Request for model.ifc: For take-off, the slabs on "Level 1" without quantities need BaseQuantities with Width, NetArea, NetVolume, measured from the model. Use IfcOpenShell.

First a look at what the model holds.

```python
import ifcopenshell
import ifcopenshell.util.element
import ifcopenshell.util.unit

model = ifcopenshell.open("model.ifc")
print(model.schema)
for unit_type in ("LENGTHUNIT", "AREAUNIT", "VOLUMEUNIT"):
    print(unit_type, ifcopenshell.util.unit.calculate_unit_scale(model, unit_type))
storey = next(s for s in model.by_type("IfcBuildingStorey") if s.Name == "Level 1")
slabs = [e for e in ifcopenshell.util.element.get_decomposition(storey) if e.is_a("IfcSlab")]
for e in sorted(slabs, key=lambda e: e.id()):
    print(e.id(), e.is_a(), e.Name, list(ifcopenshell.util.element.get_psets(e, qtos_only=True)), sep=" | ")
```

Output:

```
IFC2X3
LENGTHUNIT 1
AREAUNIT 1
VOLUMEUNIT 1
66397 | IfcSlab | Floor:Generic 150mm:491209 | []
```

```python
import ifcopenshell
import ifcopenshell.api.pset
import ifcopenshell.geom
import ifcopenshell.util.element
import ifcopenshell.util.shape
import ifcopenshell.util.unit

model = ifcopenshell.open("model.ifc")
unit_scale = ifcopenshell.util.unit.calculate_unit_scale(model)
area_scale = ifcopenshell.util.unit.calculate_unit_scale(model, "AREAUNIT")
volume_scale = ifcopenshell.util.unit.calculate_unit_scale(model, "VOLUMEUNIT")
settings = ifcopenshell.geom.settings()

storey = next(s for s in model.by_type("IfcBuildingStorey") if s.Name == "Level 1")
slabs = [e for e in ifcopenshell.util.element.get_decomposition(storey) if e.is_a("IfcSlab")]

for e in sorted(slabs, key=lambda e: e.id()):
    if ifcopenshell.util.element.get_psets(e, qtos_only=True, should_inherit=False):
        continue
    # Geometry comes back in metres, in the element's own axes.
    shape = ifcopenshell.geom.create_shape(settings, e)
    values = {
        "Width": ifcopenshell.util.shape.get_z(shape.geometry) / unit_scale,
        "NetArea": ifcopenshell.util.shape.get_footprint_area(shape.geometry) / area_scale,
        "NetVolume": ifcopenshell.util.shape.get_volume(shape.geometry) / volume_scale,
    }
    qto = ifcopenshell.api.pset.add_qto(model, product=e, name="BaseQuantities")
    ifcopenshell.api.pset.edit_qto(model, qto=qto, properties=values)
    print(e.id(), {k: round(v, 3) for k, v in values.items()})

model.write("model_rev.ifc")
```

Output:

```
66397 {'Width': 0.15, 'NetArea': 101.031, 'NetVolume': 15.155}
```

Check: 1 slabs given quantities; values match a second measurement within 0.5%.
